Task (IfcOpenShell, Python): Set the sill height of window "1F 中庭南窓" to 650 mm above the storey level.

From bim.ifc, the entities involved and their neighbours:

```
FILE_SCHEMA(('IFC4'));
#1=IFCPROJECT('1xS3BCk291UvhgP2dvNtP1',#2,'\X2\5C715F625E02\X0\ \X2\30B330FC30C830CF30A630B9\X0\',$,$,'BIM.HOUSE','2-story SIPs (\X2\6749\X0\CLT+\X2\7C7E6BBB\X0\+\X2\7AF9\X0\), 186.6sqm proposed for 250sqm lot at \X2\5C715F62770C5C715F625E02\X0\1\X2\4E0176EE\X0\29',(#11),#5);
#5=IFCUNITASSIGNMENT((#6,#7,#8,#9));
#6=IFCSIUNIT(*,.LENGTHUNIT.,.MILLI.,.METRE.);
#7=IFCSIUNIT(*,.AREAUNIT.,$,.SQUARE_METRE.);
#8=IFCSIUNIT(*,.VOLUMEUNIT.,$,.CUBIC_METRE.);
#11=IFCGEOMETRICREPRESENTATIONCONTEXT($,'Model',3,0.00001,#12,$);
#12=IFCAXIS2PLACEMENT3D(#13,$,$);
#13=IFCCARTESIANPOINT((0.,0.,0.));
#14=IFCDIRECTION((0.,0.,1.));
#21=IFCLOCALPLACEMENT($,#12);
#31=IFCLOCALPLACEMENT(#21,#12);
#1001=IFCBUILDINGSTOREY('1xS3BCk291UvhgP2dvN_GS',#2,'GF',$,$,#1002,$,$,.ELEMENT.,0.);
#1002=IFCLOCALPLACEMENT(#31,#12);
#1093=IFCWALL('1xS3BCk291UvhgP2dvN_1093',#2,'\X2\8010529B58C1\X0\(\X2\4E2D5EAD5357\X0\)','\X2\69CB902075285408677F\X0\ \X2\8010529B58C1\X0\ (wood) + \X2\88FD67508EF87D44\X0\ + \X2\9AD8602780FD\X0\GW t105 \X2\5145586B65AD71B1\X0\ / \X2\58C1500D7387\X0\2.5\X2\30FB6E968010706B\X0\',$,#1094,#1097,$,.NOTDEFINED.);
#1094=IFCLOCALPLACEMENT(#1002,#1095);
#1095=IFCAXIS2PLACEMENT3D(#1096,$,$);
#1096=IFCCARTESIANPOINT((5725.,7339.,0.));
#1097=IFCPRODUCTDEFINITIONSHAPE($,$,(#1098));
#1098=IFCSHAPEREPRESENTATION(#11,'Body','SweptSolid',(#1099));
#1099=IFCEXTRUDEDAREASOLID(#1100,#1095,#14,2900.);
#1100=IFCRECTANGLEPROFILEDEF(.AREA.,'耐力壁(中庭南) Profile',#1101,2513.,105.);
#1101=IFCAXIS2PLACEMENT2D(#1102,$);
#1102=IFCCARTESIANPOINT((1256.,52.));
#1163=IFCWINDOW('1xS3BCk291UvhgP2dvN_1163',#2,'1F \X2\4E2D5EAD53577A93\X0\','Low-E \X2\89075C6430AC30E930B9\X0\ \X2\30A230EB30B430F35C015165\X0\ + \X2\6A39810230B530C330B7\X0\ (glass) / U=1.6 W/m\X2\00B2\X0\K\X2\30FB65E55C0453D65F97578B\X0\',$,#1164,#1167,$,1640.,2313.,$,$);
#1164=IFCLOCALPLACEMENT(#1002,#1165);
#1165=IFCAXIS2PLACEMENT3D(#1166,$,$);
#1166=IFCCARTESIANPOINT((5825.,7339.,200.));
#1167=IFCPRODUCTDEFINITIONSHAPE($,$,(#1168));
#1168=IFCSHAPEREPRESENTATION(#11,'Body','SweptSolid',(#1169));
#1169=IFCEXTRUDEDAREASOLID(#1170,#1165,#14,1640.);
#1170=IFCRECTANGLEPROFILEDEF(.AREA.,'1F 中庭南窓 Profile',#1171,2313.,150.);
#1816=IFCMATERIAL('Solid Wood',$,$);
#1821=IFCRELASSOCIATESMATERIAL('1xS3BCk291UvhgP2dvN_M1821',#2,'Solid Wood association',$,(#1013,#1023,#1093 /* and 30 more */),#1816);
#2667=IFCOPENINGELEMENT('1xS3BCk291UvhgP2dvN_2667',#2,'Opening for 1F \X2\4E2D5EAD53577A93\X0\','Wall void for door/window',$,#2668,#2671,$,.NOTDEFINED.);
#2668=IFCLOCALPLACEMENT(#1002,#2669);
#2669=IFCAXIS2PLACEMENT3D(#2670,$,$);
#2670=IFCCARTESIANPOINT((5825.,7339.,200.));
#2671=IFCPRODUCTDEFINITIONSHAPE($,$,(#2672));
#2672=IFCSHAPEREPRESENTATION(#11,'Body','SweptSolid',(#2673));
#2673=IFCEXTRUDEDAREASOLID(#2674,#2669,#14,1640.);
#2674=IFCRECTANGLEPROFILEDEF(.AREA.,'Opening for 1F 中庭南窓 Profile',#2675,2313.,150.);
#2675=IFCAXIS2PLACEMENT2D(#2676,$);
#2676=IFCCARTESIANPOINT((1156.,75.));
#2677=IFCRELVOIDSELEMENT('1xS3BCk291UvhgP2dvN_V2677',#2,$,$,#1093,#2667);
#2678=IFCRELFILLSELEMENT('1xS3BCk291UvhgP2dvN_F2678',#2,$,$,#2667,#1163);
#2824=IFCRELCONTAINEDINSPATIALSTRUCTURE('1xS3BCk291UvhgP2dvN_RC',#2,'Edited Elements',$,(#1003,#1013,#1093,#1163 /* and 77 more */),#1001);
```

```python
import numpy as np
import ifcopenshell
import ifcopenshell.api.geometry
import ifcopenshell.geom
import ifcopenshell.util.element
import ifcopenshell.util.placement
import ifcopenshell.util.shape
import ifcopenshell.util.unit

model = ifcopenshell.open("bim.ifc")
unit_scale = ifcopenshell.util.unit.calculate_unit_scale(model)

window = model.by_guid("1xS3BCk291UvhgP2dvN_1163")
opening = window.FillsVoids[0].RelatingOpeningElement
storey = ifcopenshell.util.element.get_container(window, ifc_class="IfcBuildingStorey")
level = ifcopenshell.util.placement.get_local_placement(storey.ObjectPlacement)[2, 3]

# The opening's origin need not be at the sill, so measure its lowest point.
shape = ifcopenshell.geom.create_shape(ifcopenshell.geom.settings(), opening)
bottom = ifcopenshell.util.shape.get_shape_bottom_elevation(shape, shape.geometry) / unit_scale
dz = level + 0.65 / unit_scale - bottom

shift = np.array([0.0, 0.0, dz])
# The window is not placed relative to its opening, so move both.
for product in (opening, window):
    matrix = ifcopenshell.util.placement.get_local_placement(product.ObjectPlacement)
    matrix[:3, 3] += shift
    ifcopenshell.api.geometry.edit_object_placement(model, product=product, matrix=matrix, is_si=False)

print(f"moved by {dz * unit_scale:+.3f} m")

model.write("bim_edited.ifc")
```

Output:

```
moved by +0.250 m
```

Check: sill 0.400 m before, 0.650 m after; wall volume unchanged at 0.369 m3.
